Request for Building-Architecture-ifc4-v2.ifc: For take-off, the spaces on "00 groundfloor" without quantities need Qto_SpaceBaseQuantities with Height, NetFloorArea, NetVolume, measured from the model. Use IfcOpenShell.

First a look at what the model holds.

```python
import ifcopenshell
import ifcopenshell.util.element
import ifcopenshell.util.unit

model = ifcopenshell.open("Building-Architecture-ifc4-v2.ifc")
print(model.schema)
for unit_type in ("LENGTHUNIT", "AREAUNIT", "VOLUMEUNIT"):
    print(unit_type, ifcopenshell.util.unit.calculate_unit_scale(model, unit_type))
storey = next(s for s in model.by_type("IfcBuildingStorey") if s.Name == "00 groundfloor")
spaces = [e for e in ifcopenshell.util.element.get_decomposition(storey) if e.is_a("IfcSpace")]
for e in sorted(spaces, key=lambda e: e.id()):
    print(e.id(), e.is_a(), e.Name, list(ifcopenshell.util.element.get_psets(e, qtos_only=True)), sep=" | ")
```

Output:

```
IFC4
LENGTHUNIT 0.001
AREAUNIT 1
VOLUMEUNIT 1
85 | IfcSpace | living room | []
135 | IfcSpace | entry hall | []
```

```python
import ifcopenshell
import ifcopenshell.api.pset
import ifcopenshell.geom
import ifcopenshell.util.element
import ifcopenshell.util.shape
import ifcopenshell.util.unit

model = ifcopenshell.open("Building-Architecture-ifc4-v2.ifc")
unit_scale = ifcopenshell.util.unit.calculate_unit_scale(model)
area_scale = ifcopenshell.util.unit.calculate_unit_scale(model, "AREAUNIT")
volume_scale = ifcopenshell.util.unit.calculate_unit_scale(model, "VOLUMEUNIT")
settings = ifcopenshell.geom.settings()

storey = next(s for s in model.by_type("IfcBuildingStorey") if s.Name == "00 groundfloor")
spaces = [e for e in ifcopenshell.util.element.get_decomposition(storey) if e.is_a("IfcSpace")]

for e in sorted(spaces, key=lambda e: e.id()):
    if ifcopenshell.util.element.get_psets(e, qtos_only=True, should_inherit=False):
        continue
    # Geometry comes back in metres, in the element's own axes.
    shape = ifcopenshell.geom.create_shape(settings, e)
    values = {
        "Height": ifcopenshell.util.shape.get_z(shape.geometry) / unit_scale,
        "NetFloorArea": ifcopenshell.util.shape.get_footprint_area(shape.geometry) / area_scale,
        "NetVolume": ifcopenshell.util.shape.get_volume(shape.geometry) / volume_scale,
    }
    qto = ifcopenshell.api.pset.add_qto(model, product=e, name="Qto_SpaceBaseQuantities")
    ifcopenshell.api.pset.edit_qto(model, qto=qto, properties=values)
    print(e.id(), {k: round(v, 3) for k, v in values.items()})

model.write("Building-Architecture-ifc4-v2-out.ifc")
```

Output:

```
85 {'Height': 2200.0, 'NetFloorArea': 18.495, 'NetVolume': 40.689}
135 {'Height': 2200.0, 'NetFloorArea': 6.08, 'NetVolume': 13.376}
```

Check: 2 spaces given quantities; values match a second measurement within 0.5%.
